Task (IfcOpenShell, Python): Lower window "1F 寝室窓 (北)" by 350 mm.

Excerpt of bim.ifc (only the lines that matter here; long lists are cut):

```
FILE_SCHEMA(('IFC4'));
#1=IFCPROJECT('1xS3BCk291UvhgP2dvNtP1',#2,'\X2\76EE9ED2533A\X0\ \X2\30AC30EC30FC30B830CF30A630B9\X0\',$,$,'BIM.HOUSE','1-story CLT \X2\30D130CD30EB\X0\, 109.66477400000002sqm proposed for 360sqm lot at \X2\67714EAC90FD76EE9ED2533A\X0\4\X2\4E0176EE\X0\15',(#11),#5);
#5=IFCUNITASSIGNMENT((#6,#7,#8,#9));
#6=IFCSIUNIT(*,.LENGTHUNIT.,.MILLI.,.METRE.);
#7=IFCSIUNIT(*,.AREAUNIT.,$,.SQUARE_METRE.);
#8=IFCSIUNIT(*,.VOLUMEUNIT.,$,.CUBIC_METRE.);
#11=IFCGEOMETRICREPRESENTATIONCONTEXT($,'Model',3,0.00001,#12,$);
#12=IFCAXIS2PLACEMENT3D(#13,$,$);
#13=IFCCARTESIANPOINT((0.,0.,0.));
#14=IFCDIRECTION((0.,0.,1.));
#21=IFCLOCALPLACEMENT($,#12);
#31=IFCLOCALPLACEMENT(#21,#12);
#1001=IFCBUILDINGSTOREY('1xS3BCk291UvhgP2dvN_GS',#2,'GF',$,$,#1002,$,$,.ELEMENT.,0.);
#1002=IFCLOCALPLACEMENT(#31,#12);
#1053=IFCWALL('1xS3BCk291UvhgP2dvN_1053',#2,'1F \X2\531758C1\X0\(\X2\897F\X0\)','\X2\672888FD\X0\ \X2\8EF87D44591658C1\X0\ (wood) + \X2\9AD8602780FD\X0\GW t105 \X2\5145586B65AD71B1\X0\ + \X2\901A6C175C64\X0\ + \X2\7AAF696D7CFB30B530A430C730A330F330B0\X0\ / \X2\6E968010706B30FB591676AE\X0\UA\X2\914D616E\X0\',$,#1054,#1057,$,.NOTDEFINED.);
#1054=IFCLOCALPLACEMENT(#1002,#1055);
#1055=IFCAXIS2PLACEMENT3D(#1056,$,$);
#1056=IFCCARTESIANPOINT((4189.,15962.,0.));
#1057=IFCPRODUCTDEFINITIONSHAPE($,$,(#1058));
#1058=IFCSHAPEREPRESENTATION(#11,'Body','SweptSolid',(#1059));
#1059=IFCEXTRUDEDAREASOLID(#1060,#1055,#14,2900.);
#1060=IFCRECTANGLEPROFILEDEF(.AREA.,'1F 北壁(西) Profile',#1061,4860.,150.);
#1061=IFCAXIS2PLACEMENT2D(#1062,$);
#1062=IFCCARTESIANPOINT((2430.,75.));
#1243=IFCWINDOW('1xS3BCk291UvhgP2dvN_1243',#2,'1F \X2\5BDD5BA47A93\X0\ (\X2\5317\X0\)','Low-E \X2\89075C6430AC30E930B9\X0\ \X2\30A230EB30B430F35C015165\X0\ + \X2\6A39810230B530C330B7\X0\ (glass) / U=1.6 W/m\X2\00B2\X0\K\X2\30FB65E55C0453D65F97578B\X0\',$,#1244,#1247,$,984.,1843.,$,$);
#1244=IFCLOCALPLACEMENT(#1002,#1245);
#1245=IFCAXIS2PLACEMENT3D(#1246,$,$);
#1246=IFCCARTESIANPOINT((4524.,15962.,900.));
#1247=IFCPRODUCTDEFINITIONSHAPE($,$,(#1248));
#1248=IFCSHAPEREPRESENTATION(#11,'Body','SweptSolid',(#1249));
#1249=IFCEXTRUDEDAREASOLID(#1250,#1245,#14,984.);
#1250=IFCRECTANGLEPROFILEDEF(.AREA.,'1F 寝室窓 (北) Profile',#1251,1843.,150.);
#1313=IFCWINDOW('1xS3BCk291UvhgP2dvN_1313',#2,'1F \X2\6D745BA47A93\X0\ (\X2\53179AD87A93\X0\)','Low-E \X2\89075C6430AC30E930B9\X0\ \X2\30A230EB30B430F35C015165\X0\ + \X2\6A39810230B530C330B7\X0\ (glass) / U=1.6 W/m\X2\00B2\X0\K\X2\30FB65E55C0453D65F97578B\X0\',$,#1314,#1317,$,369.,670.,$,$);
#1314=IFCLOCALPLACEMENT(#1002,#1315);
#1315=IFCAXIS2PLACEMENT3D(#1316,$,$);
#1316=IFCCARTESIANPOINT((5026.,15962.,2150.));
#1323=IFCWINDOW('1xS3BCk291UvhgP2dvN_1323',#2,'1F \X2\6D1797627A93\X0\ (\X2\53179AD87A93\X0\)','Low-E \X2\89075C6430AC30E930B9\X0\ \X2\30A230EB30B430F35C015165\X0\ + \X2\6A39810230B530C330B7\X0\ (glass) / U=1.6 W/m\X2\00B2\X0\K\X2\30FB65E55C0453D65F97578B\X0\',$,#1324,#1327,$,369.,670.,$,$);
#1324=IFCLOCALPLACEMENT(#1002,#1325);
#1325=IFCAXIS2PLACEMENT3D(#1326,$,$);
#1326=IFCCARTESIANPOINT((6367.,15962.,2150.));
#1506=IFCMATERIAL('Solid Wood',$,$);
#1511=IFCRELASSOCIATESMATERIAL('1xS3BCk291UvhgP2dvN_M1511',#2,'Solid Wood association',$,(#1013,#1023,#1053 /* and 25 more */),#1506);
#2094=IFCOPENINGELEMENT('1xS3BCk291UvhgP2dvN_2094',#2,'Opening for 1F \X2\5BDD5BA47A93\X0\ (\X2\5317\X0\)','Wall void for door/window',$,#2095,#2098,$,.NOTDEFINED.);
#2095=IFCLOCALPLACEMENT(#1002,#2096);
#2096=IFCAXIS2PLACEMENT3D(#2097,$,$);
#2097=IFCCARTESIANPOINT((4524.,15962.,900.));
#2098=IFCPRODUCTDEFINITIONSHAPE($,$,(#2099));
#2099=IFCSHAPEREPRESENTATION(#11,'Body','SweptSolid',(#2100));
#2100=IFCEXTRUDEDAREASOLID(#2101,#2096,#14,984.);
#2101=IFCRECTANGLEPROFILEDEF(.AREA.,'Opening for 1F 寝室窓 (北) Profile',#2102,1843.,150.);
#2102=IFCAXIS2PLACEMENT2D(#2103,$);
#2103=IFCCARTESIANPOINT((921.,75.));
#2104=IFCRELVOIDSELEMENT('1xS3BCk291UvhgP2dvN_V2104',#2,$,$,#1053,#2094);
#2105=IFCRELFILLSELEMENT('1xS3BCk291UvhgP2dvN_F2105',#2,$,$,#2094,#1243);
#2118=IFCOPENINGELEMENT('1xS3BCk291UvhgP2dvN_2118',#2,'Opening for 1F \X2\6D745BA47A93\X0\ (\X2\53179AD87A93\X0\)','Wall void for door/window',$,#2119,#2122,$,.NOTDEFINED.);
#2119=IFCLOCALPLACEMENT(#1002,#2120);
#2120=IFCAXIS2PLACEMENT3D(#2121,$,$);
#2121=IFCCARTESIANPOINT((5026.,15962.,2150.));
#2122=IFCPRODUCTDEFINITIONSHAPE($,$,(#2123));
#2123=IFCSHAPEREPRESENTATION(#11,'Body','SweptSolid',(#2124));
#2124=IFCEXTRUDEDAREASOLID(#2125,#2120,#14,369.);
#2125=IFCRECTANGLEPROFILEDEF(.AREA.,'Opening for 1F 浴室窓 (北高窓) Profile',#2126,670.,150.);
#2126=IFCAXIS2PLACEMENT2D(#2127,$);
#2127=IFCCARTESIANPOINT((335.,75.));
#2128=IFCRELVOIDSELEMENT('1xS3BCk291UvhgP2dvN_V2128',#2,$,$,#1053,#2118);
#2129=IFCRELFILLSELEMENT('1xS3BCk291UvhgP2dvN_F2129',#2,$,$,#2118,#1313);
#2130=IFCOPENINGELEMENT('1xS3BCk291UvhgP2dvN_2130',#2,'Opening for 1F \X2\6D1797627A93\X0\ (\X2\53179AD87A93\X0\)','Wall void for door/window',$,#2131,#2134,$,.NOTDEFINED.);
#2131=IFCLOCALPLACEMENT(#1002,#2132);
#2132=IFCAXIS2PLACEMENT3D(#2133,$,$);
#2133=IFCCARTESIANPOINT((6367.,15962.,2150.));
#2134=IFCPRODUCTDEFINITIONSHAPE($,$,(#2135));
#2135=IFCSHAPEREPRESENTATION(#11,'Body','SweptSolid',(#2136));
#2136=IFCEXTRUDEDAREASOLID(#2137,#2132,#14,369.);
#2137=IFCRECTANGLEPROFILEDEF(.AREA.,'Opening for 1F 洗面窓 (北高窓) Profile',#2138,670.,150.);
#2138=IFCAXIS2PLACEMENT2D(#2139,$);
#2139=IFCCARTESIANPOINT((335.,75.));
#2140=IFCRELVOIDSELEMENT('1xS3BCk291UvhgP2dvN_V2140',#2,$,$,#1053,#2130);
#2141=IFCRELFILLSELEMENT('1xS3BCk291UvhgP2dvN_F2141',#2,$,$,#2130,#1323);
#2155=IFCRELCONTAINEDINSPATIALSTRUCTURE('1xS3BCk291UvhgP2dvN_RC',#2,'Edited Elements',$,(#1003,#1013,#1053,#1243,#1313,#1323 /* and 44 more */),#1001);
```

```python
import numpy as np
import ifcopenshell
import ifcopenshell.api.geometry
import ifcopenshell.util.placement
import ifcopenshell.util.unit

model = ifcopenshell.open("bim.ifc")
unit_scale = ifcopenshell.util.unit.calculate_unit_scale(model)

window = model.by_guid("1xS3BCk291UvhgP2dvN_1243")
opening = window.FillsVoids[0].RelatingOpeningElement
dz = -0.35 / unit_scale

shift = np.array([0.0, 0.0, dz])
# The window is not placed relative to its opening, so move both.
for product in (opening, window):
    matrix = ifcopenshell.util.placement.get_local_placement(product.ObjectPlacement)
    matrix[:3, 3] += shift
    ifcopenshell.api.geometry.edit_object_placement(model, product=product, matrix=matrix, is_si=False)

print(f"moved by {dz * unit_scale:+.3f} m")

model.write("bim_v2.ifc")
```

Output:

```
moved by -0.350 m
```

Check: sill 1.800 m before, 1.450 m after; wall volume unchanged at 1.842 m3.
